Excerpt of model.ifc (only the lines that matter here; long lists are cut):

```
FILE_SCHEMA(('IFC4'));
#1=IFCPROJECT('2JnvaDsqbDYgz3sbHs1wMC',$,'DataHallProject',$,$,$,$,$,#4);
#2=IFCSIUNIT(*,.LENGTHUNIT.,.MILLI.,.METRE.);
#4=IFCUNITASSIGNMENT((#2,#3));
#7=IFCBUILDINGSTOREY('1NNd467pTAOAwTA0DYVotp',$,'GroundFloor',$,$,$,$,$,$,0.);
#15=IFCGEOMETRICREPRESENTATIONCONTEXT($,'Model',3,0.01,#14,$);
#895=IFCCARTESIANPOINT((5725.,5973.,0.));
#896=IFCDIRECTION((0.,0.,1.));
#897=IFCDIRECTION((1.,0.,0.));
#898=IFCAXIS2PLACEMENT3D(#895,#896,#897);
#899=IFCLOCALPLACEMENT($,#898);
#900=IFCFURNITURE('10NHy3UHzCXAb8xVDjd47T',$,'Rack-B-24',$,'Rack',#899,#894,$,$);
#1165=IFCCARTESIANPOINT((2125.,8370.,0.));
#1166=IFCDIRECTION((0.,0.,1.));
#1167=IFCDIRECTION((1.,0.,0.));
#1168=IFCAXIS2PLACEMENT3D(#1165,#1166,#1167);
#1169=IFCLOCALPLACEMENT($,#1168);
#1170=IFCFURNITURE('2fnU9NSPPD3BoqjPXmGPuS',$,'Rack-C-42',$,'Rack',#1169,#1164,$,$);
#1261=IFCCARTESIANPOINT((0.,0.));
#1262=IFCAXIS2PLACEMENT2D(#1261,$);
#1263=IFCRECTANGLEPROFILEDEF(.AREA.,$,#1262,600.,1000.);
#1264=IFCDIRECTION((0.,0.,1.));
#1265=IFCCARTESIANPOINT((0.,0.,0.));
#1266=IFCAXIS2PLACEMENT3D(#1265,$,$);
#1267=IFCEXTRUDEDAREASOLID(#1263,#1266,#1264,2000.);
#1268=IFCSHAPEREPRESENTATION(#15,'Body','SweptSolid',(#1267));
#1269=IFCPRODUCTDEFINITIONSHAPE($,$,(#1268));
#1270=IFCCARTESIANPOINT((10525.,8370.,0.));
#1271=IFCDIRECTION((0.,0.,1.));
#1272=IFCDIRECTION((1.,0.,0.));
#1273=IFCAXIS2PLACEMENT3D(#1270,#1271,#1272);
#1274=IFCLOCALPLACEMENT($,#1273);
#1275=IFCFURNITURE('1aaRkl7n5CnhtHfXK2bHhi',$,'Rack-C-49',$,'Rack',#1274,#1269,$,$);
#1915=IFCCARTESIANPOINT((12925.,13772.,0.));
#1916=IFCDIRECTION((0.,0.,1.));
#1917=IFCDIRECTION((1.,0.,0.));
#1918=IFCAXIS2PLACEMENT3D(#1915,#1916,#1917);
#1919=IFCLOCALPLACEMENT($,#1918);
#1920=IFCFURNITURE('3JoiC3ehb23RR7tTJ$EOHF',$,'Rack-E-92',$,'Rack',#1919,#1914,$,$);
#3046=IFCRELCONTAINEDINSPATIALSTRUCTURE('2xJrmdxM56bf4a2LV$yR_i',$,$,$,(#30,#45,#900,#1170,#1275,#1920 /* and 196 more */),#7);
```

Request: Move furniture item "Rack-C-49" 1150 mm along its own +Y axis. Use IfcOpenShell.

```python
import ifcopenshell
import ifcopenshell.api.geometry
import ifcopenshell.util.placement
import ifcopenshell.util.unit

model = ifcopenshell.open("model.ifc")
unit_scale = ifcopenshell.util.unit.calculate_unit_scale(model)

item = model.by_guid("1aaRkl7n5CnhtHfXK2bHhi")
matrix = ifcopenshell.util.placement.get_local_placement(item.ObjectPlacement)
matrix[:3, 3] += matrix[:3, 1] * 1.15 / unit_scale
ifcopenshell.api.geometry.edit_object_placement(model, product=item, matrix=matrix, is_si=False)

print(ifcopenshell.util.placement.get_local_placement(item.ObjectPlacement).round(3) + 0.0)

model.write("model_v2.ifc")
```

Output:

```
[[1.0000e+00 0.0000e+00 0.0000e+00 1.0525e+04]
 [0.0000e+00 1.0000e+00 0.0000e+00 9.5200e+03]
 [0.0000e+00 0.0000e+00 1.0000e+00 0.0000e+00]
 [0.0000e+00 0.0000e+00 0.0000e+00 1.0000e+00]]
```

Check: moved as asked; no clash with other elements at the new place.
